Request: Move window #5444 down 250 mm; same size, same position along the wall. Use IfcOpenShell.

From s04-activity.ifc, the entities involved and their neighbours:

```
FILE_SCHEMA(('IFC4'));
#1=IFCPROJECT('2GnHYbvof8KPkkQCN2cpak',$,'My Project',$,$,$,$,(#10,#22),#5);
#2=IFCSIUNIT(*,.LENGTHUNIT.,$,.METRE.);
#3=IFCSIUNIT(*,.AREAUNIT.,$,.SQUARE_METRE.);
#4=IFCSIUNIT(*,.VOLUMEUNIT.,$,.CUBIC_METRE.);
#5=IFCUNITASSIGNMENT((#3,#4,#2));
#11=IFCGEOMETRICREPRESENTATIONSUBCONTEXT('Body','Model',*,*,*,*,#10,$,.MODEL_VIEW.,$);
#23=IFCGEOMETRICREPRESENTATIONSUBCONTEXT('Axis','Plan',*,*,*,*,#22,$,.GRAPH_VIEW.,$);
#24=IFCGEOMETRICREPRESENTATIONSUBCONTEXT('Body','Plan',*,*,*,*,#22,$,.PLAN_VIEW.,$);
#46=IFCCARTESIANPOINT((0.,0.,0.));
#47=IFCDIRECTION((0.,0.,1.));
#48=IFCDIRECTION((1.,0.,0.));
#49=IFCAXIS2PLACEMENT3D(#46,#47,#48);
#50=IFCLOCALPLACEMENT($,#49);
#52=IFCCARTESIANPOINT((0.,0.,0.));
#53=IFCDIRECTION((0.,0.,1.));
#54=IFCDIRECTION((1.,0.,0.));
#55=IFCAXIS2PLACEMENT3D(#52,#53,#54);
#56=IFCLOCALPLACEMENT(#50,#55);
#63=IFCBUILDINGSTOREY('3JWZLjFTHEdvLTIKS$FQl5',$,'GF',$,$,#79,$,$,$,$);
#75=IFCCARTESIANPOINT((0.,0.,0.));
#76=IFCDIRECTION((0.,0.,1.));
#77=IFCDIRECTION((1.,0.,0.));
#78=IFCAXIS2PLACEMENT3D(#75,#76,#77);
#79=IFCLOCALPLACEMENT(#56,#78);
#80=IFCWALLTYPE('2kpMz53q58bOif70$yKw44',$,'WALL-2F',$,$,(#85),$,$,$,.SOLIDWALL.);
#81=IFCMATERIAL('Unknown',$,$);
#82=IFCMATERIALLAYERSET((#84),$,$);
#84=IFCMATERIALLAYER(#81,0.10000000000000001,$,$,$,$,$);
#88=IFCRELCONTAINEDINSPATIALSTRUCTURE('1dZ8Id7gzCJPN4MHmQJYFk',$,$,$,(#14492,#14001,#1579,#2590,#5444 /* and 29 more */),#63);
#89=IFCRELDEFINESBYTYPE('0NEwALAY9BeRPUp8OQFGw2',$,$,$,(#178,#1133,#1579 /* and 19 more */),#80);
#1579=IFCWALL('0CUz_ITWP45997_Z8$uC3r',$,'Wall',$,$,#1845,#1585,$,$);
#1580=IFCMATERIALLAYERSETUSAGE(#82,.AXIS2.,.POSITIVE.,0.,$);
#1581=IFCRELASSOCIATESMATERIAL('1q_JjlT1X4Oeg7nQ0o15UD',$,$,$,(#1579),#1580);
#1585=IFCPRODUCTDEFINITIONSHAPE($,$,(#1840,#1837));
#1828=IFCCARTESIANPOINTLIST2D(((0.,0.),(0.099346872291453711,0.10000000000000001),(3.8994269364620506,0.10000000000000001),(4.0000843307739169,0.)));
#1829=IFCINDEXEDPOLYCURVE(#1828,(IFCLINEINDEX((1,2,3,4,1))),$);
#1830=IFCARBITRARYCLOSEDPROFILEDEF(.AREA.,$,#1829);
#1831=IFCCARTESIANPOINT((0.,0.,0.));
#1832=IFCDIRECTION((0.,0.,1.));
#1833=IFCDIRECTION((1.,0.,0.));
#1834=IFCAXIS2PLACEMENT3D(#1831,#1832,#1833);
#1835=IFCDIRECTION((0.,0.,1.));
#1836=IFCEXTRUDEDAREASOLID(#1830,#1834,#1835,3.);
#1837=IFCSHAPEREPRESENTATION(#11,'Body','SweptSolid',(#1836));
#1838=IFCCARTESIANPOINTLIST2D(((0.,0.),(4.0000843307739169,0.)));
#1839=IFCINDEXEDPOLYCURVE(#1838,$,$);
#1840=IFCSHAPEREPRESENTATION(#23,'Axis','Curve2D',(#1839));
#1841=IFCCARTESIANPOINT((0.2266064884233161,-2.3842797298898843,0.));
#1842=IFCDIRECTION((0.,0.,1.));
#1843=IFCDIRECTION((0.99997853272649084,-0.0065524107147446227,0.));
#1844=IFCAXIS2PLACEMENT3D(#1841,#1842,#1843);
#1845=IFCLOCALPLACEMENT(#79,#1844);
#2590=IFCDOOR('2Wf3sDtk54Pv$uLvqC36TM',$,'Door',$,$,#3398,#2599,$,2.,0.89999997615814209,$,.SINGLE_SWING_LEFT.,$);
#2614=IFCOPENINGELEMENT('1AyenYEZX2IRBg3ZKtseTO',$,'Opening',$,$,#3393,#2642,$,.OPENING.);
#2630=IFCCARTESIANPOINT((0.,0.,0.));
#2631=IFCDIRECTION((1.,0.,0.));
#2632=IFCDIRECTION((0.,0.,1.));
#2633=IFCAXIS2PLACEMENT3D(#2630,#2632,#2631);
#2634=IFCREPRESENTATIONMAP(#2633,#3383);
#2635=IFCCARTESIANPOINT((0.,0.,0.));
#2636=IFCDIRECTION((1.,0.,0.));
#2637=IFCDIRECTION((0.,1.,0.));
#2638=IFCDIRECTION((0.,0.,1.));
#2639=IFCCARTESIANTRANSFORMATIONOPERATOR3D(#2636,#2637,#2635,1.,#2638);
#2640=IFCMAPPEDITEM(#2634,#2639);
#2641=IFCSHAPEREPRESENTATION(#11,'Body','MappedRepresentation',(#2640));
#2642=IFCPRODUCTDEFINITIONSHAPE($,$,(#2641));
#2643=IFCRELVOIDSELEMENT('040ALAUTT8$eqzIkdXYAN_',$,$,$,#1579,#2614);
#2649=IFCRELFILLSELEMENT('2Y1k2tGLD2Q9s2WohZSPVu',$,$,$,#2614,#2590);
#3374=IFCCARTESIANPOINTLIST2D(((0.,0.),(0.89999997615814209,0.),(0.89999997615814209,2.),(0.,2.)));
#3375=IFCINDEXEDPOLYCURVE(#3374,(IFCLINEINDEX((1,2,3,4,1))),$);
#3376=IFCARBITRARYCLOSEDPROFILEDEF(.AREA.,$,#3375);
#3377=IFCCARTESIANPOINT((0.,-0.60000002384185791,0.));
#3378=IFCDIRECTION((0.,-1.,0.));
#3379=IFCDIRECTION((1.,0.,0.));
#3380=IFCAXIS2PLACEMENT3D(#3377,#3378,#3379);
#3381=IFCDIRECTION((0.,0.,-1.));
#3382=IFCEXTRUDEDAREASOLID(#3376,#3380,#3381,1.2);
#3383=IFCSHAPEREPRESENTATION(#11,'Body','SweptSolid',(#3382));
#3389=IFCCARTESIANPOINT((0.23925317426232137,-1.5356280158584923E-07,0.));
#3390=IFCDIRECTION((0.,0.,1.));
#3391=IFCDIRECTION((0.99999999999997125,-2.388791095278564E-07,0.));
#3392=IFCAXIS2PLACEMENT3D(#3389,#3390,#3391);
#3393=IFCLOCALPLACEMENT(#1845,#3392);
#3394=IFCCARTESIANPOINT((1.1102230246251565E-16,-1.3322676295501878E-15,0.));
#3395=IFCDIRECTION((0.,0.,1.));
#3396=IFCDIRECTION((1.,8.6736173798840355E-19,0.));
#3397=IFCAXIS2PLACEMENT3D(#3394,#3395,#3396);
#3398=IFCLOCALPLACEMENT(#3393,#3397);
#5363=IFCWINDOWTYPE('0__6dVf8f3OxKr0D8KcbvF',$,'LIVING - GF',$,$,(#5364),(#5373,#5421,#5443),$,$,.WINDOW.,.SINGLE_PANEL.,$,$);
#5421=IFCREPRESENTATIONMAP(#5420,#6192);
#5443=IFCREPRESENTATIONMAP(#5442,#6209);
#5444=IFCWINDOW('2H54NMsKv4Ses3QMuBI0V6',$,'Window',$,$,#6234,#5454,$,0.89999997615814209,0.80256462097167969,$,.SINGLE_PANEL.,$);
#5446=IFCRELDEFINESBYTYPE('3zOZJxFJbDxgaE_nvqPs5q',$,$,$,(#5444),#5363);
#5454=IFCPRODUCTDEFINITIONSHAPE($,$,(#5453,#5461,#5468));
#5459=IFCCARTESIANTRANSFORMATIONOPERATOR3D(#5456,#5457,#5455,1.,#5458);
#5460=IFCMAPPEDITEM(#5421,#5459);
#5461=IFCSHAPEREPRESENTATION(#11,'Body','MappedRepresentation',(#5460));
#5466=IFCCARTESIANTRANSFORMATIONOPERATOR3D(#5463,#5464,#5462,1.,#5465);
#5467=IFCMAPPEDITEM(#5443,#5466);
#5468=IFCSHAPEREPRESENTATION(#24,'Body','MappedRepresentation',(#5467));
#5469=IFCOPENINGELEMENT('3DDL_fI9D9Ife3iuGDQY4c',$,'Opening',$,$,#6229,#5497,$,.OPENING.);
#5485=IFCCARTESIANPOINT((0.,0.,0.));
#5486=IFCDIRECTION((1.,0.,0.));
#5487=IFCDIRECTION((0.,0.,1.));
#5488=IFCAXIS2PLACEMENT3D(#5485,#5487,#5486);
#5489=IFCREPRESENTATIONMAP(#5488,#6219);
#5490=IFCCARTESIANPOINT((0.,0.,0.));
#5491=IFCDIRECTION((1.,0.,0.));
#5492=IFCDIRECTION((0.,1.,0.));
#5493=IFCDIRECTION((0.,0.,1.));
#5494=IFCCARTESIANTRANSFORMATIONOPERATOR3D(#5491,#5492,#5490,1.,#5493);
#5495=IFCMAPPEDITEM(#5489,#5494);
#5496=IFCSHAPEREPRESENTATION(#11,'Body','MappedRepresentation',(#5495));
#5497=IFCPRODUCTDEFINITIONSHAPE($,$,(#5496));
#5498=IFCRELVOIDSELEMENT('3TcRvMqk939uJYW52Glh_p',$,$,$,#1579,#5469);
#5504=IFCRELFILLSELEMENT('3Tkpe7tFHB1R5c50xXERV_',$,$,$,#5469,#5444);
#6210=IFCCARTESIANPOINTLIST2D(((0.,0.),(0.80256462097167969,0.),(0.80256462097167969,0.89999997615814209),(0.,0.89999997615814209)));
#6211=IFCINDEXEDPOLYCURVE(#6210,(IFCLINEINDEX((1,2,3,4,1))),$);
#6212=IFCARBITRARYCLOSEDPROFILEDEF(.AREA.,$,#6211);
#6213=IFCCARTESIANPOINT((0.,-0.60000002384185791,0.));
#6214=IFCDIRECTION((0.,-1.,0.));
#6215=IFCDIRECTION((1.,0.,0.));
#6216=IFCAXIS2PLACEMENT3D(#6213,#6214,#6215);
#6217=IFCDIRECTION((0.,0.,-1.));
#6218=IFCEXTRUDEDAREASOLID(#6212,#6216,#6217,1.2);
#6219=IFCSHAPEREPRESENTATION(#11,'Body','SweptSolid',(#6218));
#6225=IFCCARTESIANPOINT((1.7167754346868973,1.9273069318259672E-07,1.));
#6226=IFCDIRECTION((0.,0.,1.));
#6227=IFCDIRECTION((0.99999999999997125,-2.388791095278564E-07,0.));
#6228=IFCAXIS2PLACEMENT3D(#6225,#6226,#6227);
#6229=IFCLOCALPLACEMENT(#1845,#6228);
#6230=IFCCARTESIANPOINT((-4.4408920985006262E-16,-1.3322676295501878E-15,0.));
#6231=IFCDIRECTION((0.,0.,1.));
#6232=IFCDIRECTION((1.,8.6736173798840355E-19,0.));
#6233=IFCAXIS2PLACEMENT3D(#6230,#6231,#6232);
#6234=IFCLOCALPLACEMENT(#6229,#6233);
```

```python
import numpy as np
import ifcopenshell
import ifcopenshell.api.geometry
import ifcopenshell.util.placement
import ifcopenshell.util.unit

model = ifcopenshell.open("s04-activity.ifc")
unit_scale = ifcopenshell.util.unit.calculate_unit_scale(model)

window = model.by_guid("2H54NMsKv4Ses3QMuBI0V6")
opening = window.FillsVoids[0].RelatingOpeningElement
dz = -0.25 / unit_scale

shift = np.array([0.0, 0.0, dz])
# The window is placed relative to its opening, so it follows when the opening moves.
matrix = ifcopenshell.util.placement.get_local_placement(opening.ObjectPlacement)
matrix[:3, 3] += shift
ifcopenshell.api.geometry.edit_object_placement(
    model, product=opening, matrix=matrix, is_si=False, should_transform_children=True
)

print(f"moved by {dz * unit_scale:+.3f} m")

model.write("s04-activity_updated.ifc")
```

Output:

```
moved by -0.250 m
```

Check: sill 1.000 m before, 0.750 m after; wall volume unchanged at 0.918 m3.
